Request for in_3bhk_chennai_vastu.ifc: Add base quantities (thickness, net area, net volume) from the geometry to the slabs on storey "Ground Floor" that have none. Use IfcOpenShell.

First a look at what the model holds.

```python
import ifcopenshell
import ifcopenshell.util.element
import ifcopenshell.util.unit

model = ifcopenshell.open("in_3bhk_chennai_vastu.ifc")
print(model.schema)
for unit_type in ("LENGTHUNIT", "AREAUNIT", "VOLUMEUNIT"):
    print(unit_type, ifcopenshell.util.unit.calculate_unit_scale(model, unit_type))
storey = next(s for s in model.by_type("IfcBuildingStorey") if s.Name == "Ground Floor")
slabs = [e for e in ifcopenshell.util.element.get_decomposition(storey) if e.is_a("IfcSlab")]
for e in sorted(slabs, key=lambda e: e.id()):
    print(e.id(), e.is_a(), e.Name, list(ifcopenshell.util.element.get_psets(e, qtos_only=True)), sep=" | ")
```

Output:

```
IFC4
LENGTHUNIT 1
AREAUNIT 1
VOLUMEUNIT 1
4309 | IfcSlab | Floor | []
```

```python
import ifcopenshell
import ifcopenshell.api.pset
import ifcopenshell.geom
import ifcopenshell.util.element
import ifcopenshell.util.shape
import ifcopenshell.util.unit

model = ifcopenshell.open("in_3bhk_chennai_vastu.ifc")
unit_scale = ifcopenshell.util.unit.calculate_unit_scale(model)
area_scale = ifcopenshell.util.unit.calculate_unit_scale(model, "AREAUNIT")
volume_scale = ifcopenshell.util.unit.calculate_unit_scale(model, "VOLUMEUNIT")
settings = ifcopenshell.geom.settings()

storey = next(s for s in model.by_type("IfcBuildingStorey") if s.Name == "Ground Floor")
slabs = [e for e in ifcopenshell.util.element.get_decomposition(storey) if e.is_a("IfcSlab")]

for e in sorted(slabs, key=lambda e: e.id()):
    if ifcopenshell.util.element.get_psets(e, qtos_only=True, should_inherit=False):
        continue
    # Geometry comes back in metres, in the element's own axes.
    shape = ifcopenshell.geom.create_shape(settings, e)
    values = {
        "Width": ifcopenshell.util.shape.get_z(shape.geometry) / unit_scale,
        "NetArea": ifcopenshell.util.shape.get_footprint_area(shape.geometry) / area_scale,
        "NetVolume": ifcopenshell.util.shape.get_volume(shape.geometry) / volume_scale,
    }
    qto = ifcopenshell.api.pset.add_qto(model, product=e, name="Qto_SlabBaseQuantities")
    ifcopenshell.api.pset.edit_qto(model, qto=qto, properties=values)
    print(e.id(), {k: round(v, 3) for k, v in values.items()})

model.write("in_3bhk_chennai_vastu_v2.ifc")
```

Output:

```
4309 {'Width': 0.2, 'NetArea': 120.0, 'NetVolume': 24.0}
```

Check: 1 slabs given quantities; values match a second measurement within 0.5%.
